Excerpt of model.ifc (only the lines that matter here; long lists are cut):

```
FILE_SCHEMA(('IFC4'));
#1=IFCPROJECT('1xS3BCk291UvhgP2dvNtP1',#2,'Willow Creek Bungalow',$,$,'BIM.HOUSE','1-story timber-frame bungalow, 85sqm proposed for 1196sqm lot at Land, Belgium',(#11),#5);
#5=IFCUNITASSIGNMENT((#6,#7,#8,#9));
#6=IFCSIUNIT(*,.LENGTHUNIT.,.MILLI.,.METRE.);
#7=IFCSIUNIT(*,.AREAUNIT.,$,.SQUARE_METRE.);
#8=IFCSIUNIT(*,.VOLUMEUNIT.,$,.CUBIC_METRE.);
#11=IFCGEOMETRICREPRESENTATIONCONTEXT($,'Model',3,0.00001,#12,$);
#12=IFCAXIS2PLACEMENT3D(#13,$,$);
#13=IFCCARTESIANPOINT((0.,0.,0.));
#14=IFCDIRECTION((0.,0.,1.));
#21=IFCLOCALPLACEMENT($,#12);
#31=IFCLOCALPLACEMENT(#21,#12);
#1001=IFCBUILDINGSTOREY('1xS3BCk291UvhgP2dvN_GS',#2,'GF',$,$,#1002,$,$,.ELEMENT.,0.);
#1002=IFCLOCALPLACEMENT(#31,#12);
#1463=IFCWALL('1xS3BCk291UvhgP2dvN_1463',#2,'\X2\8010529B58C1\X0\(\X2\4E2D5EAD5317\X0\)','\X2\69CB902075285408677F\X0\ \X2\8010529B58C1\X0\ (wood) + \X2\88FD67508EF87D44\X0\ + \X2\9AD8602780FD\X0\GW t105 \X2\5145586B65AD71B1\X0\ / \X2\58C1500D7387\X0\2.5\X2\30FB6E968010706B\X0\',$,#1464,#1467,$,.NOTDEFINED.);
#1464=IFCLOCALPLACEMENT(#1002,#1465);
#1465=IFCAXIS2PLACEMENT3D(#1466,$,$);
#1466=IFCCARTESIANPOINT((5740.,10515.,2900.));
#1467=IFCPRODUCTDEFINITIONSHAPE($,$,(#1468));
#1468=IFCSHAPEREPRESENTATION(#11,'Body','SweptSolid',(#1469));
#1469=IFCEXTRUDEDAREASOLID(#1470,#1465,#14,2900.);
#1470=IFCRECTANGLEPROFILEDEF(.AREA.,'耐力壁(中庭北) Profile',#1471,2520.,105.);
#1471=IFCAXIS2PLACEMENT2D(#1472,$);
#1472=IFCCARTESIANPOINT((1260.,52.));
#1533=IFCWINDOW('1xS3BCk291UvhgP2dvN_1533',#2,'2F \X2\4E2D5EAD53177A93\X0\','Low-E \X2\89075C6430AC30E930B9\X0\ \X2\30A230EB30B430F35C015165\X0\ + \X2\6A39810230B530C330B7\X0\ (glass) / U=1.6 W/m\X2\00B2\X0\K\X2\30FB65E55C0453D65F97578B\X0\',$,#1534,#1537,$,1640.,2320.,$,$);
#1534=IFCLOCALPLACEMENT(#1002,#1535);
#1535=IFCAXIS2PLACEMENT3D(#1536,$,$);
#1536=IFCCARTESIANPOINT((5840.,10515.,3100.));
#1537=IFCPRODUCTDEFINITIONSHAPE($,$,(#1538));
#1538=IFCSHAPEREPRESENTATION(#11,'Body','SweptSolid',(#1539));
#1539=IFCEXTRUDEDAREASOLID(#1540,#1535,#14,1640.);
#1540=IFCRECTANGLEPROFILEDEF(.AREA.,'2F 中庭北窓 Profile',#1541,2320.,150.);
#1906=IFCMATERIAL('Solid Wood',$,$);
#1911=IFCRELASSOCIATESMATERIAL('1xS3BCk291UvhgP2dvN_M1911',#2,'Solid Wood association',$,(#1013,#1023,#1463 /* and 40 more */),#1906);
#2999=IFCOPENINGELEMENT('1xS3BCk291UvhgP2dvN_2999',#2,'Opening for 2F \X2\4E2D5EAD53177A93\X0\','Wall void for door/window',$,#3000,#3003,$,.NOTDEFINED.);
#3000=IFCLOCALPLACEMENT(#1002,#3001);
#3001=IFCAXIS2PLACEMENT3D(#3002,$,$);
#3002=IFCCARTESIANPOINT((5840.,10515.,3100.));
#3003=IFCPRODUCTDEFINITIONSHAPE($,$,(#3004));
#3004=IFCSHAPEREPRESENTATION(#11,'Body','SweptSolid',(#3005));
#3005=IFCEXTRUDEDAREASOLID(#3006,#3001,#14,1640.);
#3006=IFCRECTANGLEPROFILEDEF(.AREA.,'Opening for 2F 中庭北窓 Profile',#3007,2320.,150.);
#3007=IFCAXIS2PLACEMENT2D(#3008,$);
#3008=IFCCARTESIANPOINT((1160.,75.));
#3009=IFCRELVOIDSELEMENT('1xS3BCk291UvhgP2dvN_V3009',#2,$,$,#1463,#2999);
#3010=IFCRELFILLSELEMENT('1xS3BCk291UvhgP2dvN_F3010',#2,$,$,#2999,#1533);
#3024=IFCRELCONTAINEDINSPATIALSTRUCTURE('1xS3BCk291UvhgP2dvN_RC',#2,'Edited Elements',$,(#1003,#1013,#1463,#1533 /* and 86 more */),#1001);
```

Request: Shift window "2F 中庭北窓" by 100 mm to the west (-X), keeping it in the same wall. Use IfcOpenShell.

```python
import ifcopenshell
import ifcopenshell.api.geometry
import ifcopenshell.util.placement
import ifcopenshell.util.unit

model = ifcopenshell.open("model.ifc")
unit_scale = ifcopenshell.util.unit.calculate_unit_scale(model)

window = model.by_guid("1xS3BCk291UvhgP2dvN_1533")
opening = window.FillsVoids[0].RelatingOpeningElement
wall = opening.VoidsElements[0].RelatingBuildingElement

wall_matrix = ifcopenshell.util.placement.get_local_placement(wall.ObjectPlacement)
shift = wall_matrix[:3, 0] * -0.1 / unit_scale
before = ifcopenshell.util.placement.get_local_placement(window.ObjectPlacement)[:3, 3].copy()

# The window is not placed relative to its opening, so move both.
for product in (opening, window):
    matrix = ifcopenshell.util.placement.get_local_placement(product.ObjectPlacement)
    matrix[:3, 3] += shift
    ifcopenshell.api.geometry.edit_object_placement(model, product=product, matrix=matrix, is_si=False)

after = ifcopenshell.util.placement.get_local_placement(window.ObjectPlacement)[:3, 3]
print("window moved by", (after - before).round(3) + 0.0)

model.write("model_edited.ifc")
```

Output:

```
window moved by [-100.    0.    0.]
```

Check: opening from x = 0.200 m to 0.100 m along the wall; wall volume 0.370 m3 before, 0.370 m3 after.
